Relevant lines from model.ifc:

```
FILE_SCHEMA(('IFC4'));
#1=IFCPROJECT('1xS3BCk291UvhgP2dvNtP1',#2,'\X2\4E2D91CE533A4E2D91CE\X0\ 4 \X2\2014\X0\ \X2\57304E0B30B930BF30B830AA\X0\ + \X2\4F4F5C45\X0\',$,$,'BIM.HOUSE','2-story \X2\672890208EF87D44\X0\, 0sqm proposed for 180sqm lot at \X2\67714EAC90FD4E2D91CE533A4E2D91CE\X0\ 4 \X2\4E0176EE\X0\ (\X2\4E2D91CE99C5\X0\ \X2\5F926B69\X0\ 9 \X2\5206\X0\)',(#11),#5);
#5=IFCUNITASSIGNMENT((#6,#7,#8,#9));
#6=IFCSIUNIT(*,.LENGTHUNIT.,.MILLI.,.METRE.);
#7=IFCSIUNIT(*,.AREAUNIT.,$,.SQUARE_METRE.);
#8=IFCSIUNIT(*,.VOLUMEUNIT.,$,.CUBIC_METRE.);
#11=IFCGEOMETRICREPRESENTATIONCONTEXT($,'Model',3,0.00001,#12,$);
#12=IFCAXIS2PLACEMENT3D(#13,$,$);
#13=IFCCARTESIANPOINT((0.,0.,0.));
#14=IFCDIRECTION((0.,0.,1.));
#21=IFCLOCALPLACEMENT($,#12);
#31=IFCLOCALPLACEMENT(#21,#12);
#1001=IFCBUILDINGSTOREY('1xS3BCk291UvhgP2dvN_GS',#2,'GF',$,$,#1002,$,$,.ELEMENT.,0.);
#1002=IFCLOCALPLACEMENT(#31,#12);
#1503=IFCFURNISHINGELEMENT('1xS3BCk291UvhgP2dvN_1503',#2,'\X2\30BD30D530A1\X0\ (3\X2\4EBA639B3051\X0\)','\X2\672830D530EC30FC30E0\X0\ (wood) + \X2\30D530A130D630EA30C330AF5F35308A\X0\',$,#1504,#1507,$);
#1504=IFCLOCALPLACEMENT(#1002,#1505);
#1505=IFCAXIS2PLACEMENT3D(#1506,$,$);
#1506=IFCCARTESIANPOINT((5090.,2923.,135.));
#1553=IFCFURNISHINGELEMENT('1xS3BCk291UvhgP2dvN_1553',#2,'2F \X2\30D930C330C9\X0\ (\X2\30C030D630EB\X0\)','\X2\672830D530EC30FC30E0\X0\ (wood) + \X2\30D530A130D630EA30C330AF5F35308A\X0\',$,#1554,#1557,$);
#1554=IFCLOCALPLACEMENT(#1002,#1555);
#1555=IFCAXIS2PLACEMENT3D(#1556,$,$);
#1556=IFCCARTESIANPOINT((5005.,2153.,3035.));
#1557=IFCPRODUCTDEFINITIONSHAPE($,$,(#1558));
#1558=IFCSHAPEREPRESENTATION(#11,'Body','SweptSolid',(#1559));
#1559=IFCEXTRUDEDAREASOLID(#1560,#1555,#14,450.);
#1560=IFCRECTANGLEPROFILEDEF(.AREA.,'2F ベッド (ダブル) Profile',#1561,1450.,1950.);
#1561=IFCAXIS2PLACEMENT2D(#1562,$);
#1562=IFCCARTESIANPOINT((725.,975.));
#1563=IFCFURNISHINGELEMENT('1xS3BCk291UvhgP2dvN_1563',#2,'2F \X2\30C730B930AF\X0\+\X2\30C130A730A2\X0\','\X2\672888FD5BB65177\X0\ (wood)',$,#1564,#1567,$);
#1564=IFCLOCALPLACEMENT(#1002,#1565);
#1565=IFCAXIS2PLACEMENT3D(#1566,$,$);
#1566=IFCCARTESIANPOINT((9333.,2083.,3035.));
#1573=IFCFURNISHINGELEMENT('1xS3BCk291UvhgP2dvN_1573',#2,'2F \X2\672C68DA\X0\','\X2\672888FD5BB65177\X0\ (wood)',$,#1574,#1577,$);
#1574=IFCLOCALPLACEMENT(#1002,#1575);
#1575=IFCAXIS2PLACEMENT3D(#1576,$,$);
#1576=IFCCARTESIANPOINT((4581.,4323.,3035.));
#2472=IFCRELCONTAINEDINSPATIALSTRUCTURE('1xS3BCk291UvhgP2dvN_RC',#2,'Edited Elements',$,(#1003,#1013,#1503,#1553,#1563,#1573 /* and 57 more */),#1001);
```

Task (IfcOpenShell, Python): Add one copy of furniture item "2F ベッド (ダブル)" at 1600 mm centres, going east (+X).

```python
import numpy as np
import ifcopenshell
import ifcopenshell.api.geometry
import ifcopenshell.api.root
import ifcopenshell.util.element
import ifcopenshell.util.placement
import ifcopenshell.util.unit

model = ifcopenshell.open("model.ifc")
unit_scale = ifcopenshell.util.unit.calculate_unit_scale(model)


def reuse_history(source, copy):
    """copy_class also copies each property set's owner history, people and application; keep the originals."""
    for rel in copy.IsDefinedBy:
        if rel.is_a("IfcRelDefinesByProperties") and (history := rel.RelatingPropertyDefinition.OwnerHistory):
            rel.RelatingPropertyDefinition.OwnerHistory = source.OwnerHistory
            ifcopenshell.util.element.remove_deep2(model, history)


source = model.by_guid("1xS3BCk291UvhgP2dvN_1553")
base = ifcopenshell.util.placement.get_local_placement(source.ObjectPlacement)
step = np.array([1.0, 0.0, 0.0]) * 1.6 / unit_scale

for i in range(1, 2):
    copy = ifcopenshell.api.root.copy_class(model, product=source)
    copy.Representation = ifcopenshell.util.element.copy_deep(
        model, source.Representation, exclude=["IfcGeometricRepresentationContext", "IfcRepresentationMap"]
    )
    reuse_history(source, copy)
    matrix = base.copy()
    matrix[:3, 3] += i * step
    print("added at", matrix[:3, 3].round(3) + 0.0)
    ifcopenshell.api.geometry.edit_object_placement(model, product=copy, matrix=matrix, is_si=False)

model.write("model_updated.ifc")
```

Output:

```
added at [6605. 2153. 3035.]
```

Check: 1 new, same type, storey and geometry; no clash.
